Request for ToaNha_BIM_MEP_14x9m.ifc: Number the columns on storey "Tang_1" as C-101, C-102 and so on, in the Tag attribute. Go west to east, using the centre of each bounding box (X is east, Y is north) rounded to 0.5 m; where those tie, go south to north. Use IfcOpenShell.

First a look at what the model holds.

```python
import ifcopenshell
import ifcopenshell.util.element
import ifcopenshell.util.placement

model = ifcopenshell.open("ToaNha_BIM_MEP_14x9m.ifc")
print(model.schema)
storey = next(s for s in model.by_type("IfcBuildingStorey") if s.Name == "Tang_1")
columns = [e for e in ifcopenshell.util.element.get_decomposition(storey) if e.is_a("IfcColumn")]
for e in sorted(columns, key=lambda e: e.id()):
    origin = ifcopenshell.util.placement.get_local_placement(e.ObjectPlacement)[:3, 3]
    print(e.id(), e.Tag, e.Name, origin.round(2) + 0.0, sep=" | ")
```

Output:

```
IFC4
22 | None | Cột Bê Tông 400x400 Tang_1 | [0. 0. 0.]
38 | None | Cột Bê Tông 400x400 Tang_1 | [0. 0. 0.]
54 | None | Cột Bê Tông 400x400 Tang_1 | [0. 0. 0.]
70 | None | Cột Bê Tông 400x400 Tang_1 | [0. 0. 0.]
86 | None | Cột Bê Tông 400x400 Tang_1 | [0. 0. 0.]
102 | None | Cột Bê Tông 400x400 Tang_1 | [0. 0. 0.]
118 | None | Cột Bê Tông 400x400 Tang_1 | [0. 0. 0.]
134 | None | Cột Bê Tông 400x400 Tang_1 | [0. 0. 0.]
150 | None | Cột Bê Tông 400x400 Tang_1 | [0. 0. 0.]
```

```python
import ifcopenshell
import ifcopenshell.geom
import ifcopenshell.util.element
import ifcopenshell.util.shape

model = ifcopenshell.open("ToaNha_BIM_MEP_14x9m.ifc")
settings = ifcopenshell.geom.settings()
settings.set("use-world-coords", True)


def centre(element):
    shape = ifcopenshell.geom.create_shape(settings, element)
    return ifcopenshell.util.shape.get_bbox_centroid(shape.geometry)


storey = next(s for s in model.by_type("IfcBuildingStorey") if s.Name == "Tang_1")
columns = [e for e in ifcopenshell.util.element.get_decomposition(storey) if e.is_a("IfcColumn")]

# Insertion points can sit at a corner or the storey origin, so sort by the geometry (in metres).
centres = {e: centre(e) for e in columns}
columns.sort(key=lambda e: (round(centres[e][0] / 0.5), centres[e][1]))

for i, e in enumerate(columns, start=1):
    number = f"C-1{i:02d}"
    e.Tag = number
    print(e.id(), number)

model.write("ToaNha_BIM_MEP_14x9m-out.ifc")
```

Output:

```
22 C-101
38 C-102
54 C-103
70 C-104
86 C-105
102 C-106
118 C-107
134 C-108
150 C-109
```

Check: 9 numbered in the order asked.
